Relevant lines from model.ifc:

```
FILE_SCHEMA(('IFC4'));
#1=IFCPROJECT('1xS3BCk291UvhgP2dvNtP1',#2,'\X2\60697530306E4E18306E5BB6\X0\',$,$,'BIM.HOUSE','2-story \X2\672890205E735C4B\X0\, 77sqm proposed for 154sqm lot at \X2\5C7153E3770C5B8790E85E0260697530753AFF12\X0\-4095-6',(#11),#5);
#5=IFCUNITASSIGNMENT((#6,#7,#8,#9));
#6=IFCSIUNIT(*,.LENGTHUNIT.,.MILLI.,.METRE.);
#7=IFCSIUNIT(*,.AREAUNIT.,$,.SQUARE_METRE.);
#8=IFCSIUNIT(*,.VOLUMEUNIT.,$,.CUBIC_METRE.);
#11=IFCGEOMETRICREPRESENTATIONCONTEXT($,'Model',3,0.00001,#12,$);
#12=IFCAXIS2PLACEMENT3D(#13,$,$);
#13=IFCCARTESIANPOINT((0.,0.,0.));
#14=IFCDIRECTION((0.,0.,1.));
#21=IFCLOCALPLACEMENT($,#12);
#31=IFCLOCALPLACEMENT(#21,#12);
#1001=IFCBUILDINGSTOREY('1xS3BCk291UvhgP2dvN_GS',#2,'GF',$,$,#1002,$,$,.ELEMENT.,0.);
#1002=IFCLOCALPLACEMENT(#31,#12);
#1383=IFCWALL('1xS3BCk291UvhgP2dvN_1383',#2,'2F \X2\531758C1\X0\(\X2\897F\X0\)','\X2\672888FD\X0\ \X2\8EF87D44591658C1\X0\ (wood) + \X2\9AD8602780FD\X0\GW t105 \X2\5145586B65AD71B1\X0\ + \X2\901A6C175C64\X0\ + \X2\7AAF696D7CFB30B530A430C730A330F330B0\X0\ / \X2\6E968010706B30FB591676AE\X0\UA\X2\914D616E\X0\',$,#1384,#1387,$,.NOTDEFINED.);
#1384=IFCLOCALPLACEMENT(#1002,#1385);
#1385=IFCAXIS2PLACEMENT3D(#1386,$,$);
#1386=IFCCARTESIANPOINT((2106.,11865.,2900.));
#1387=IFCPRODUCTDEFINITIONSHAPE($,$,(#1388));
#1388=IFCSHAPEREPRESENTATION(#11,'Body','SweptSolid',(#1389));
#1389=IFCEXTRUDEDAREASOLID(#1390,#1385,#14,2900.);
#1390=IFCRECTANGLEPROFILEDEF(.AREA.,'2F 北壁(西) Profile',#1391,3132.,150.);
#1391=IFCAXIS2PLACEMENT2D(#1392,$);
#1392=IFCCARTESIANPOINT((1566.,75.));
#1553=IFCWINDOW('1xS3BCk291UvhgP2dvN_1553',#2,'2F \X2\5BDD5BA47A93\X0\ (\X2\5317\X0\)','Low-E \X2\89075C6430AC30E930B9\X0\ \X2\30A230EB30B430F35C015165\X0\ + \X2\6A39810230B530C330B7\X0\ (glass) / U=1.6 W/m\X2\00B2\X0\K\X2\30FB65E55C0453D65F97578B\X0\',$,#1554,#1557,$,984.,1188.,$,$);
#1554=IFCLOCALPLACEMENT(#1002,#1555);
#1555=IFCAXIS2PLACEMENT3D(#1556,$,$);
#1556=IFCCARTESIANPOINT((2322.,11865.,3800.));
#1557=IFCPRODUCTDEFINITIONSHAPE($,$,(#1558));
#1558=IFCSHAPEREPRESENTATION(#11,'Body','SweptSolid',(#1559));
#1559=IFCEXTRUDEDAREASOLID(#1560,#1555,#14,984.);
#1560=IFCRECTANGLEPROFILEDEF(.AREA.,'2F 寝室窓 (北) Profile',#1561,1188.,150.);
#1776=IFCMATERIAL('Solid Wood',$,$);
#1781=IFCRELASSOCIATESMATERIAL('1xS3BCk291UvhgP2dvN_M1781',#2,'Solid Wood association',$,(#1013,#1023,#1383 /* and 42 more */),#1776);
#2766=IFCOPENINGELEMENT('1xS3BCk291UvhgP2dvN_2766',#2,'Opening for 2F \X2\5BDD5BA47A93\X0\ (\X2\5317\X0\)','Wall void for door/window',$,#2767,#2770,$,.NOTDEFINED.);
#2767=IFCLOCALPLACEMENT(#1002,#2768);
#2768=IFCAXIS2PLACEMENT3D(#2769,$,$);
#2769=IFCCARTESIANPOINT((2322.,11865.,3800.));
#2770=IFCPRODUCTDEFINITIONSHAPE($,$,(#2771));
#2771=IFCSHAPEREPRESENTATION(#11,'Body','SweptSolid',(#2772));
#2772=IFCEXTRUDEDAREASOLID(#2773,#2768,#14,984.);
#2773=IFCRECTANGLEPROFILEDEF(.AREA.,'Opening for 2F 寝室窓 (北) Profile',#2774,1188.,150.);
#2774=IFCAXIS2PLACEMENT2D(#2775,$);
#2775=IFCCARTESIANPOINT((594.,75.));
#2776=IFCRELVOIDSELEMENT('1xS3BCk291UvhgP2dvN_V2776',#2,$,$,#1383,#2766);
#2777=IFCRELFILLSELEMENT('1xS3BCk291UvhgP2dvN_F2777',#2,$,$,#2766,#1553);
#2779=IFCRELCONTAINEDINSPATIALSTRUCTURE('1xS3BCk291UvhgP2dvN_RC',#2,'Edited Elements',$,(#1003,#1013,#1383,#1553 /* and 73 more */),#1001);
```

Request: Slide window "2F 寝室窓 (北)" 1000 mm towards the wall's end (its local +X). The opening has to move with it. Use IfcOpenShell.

```python
import ifcopenshell
import ifcopenshell.api.geometry
import ifcopenshell.util.placement
import ifcopenshell.util.unit

model = ifcopenshell.open("model.ifc")
unit_scale = ifcopenshell.util.unit.calculate_unit_scale(model)

window = model.by_id(1553)
opening = window.FillsVoids[0].RelatingOpeningElement
wall = opening.VoidsElements[0].RelatingBuildingElement

wall_matrix = ifcopenshell.util.placement.get_local_placement(wall.ObjectPlacement)
shift = wall_matrix[:3, 0] * 1 / unit_scale
before = ifcopenshell.util.placement.get_local_placement(window.ObjectPlacement)[:3, 3].copy()

# The window is not placed relative to its opening, so move both.
for product in (opening, window):
    matrix = ifcopenshell.util.placement.get_local_placement(product.ObjectPlacement)
    matrix[:3, 3] += shift
    ifcopenshell.api.geometry.edit_object_placement(model, product=product, matrix=matrix, is_si=False)

after = ifcopenshell.util.placement.get_local_placement(window.ObjectPlacement)[:3, 3]
print("window moved by", (after - before).round(3) + 0.0)

model.write("model_updated.ifc")
```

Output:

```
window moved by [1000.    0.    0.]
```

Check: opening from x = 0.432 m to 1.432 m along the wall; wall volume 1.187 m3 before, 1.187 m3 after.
